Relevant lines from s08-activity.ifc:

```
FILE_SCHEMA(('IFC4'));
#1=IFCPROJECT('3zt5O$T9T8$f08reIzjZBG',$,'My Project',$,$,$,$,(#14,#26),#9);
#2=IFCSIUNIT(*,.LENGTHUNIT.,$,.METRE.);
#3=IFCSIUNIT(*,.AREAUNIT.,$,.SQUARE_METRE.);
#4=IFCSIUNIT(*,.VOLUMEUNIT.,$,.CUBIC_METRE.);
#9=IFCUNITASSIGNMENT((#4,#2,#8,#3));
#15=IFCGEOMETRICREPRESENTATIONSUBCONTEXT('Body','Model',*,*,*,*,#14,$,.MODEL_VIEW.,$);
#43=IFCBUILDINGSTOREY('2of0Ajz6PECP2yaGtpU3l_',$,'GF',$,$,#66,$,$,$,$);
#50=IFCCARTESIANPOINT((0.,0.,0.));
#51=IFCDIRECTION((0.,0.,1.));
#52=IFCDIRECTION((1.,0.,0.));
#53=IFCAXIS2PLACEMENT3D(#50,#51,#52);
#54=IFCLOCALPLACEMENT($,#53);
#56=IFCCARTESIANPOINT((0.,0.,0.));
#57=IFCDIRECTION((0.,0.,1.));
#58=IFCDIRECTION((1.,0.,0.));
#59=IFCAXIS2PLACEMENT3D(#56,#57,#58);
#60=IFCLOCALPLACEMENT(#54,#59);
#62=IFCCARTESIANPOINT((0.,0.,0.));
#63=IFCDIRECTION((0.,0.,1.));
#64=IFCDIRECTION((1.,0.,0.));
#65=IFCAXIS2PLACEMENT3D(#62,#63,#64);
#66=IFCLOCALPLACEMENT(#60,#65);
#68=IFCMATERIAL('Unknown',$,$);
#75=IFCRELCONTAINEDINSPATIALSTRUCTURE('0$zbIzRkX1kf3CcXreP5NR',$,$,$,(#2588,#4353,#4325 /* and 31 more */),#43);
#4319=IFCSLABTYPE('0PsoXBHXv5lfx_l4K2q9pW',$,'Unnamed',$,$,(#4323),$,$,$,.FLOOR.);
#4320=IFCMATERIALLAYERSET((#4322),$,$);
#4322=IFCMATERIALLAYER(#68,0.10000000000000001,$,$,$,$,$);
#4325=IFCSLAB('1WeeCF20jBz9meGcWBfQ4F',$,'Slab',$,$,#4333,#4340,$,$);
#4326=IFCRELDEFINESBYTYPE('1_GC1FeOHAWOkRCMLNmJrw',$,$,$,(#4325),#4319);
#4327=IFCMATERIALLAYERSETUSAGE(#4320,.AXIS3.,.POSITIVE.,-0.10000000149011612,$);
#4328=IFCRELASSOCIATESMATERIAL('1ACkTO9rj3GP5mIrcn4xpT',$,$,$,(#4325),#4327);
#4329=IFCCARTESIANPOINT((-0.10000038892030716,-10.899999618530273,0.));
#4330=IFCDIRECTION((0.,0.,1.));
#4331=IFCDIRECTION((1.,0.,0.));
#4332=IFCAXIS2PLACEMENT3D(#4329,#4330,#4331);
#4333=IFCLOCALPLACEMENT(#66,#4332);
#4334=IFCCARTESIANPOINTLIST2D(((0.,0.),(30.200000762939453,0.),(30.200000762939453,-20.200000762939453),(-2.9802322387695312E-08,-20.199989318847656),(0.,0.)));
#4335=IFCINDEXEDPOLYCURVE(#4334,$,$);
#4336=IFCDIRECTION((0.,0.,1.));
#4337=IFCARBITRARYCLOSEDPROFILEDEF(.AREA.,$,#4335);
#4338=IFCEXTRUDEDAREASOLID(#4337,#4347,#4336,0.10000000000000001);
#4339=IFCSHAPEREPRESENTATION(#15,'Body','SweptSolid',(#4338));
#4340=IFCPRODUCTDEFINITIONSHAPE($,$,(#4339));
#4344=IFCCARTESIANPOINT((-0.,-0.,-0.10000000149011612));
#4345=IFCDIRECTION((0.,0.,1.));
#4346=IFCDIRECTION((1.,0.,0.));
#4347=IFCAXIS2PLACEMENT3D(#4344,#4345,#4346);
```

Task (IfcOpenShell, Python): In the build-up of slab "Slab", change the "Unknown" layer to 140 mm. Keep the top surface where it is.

```python
import ifcopenshell
import ifcopenshell.util.element
import ifcopenshell.util.representation

model = ifcopenshell.open("s08-activity.ifc")

layer_set = model.by_id(4320)
layer = next(l for l in layer_set.MaterialLayers if l.Material and l.Material.Name == "Unknown")
change = 0.14 - layer.LayerThickness
layer.LayerThickness += change

# Geometry does not follow the layer set by itself.
slabs = [e for e in ifcopenshell.util.element.get_elements_by_material(model, layer_set) if e.is_a("IfcSlab")]
for slab in sorted(slabs, key=lambda e: e.id()):
    body = ifcopenshell.util.representation.get_representation(slab, "Model", "Body")
    solid = body.Items[0]
    old_depth = solid.Depth
    solid.Depth += change
    # Extruded upwards: lower the start of the extrusion so the top stays.
    x, y, z = solid.Position.Location.Coordinates
    solid.Position.Location = model.createIfcCartesianPoint((x, y, z - change))
    print(slab.id(), f"{old_depth:g} -> {solid.Depth:g}")

# The layers are counted up from the underside, which has moved.
for usage in {ifcopenshell.util.element.get_material(slab) for slab in slabs}:
    usage.OffsetFromReferenceLine -= change

model.write("s08-activity-out.ifc")
```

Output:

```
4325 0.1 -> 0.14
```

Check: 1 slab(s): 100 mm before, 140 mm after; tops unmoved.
